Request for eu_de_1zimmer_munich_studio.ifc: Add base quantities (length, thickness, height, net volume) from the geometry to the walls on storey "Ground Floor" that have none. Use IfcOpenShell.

First a look at what the model holds.

```python
import ifcopenshell
import ifcopenshell.util.element
import ifcopenshell.util.unit

model = ifcopenshell.open("eu_de_1zimmer_munich_studio.ifc")
print(model.schema)
for unit_type in ("LENGTHUNIT", "AREAUNIT", "VOLUMEUNIT"):
    print(unit_type, ifcopenshell.util.unit.calculate_unit_scale(model, unit_type))
storey = next(s for s in model.by_type("IfcBuildingStorey") if s.Name == "Ground Floor")
walls = [e for e in ifcopenshell.util.element.get_decomposition(storey) if e.is_a("IfcWall")]
for e in sorted(walls, key=lambda e: e.id()):
    print(e.id(), e.is_a(), e.Name, list(ifcopenshell.util.element.get_psets(e, qtos_only=True)), sep=" | ")
```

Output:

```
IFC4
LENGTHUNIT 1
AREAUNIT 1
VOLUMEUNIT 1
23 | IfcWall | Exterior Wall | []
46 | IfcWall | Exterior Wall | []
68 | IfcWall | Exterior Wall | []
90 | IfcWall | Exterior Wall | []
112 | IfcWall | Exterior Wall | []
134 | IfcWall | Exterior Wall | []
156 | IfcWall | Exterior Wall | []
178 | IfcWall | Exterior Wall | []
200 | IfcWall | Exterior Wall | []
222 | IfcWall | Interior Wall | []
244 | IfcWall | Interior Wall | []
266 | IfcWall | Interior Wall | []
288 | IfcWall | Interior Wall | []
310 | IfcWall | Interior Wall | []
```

```python
import ifcopenshell
import ifcopenshell.api.pset
import ifcopenshell.geom
import ifcopenshell.util.element
import ifcopenshell.util.shape
import ifcopenshell.util.unit

model = ifcopenshell.open("eu_de_1zimmer_munich_studio.ifc")
unit_scale = ifcopenshell.util.unit.calculate_unit_scale(model)
volume_scale = ifcopenshell.util.unit.calculate_unit_scale(model, "VOLUMEUNIT")
settings = ifcopenshell.geom.settings()

storey = next(s for s in model.by_type("IfcBuildingStorey") if s.Name == "Ground Floor")
walls = [e for e in ifcopenshell.util.element.get_decomposition(storey) if e.is_a("IfcWall")]

for e in sorted(walls, key=lambda e: e.id()):
    if ifcopenshell.util.element.get_psets(e, qtos_only=True, should_inherit=False):
        continue
    # Geometry comes back in metres, in the element's own axes.
    shape = ifcopenshell.geom.create_shape(settings, e)
    values = {
        "Length": ifcopenshell.util.shape.get_x(shape.geometry) / unit_scale,
        "Width": ifcopenshell.util.shape.get_y(shape.geometry) / unit_scale,
        "Height": ifcopenshell.util.shape.get_z(shape.geometry) / unit_scale,
        "NetVolume": ifcopenshell.util.shape.get_volume(shape.geometry) / volume_scale,
    }
    qto = ifcopenshell.api.pset.add_qto(model, product=e, name="Qto_WallBaseQuantities")
    ifcopenshell.api.pset.edit_qto(model, qto=qto, properties=values)
    print(e.id(), {k: round(v, 3) for k, v in values.items()})

model.write("eu_de_1zimmer_munich_studio_edited.ifc")
```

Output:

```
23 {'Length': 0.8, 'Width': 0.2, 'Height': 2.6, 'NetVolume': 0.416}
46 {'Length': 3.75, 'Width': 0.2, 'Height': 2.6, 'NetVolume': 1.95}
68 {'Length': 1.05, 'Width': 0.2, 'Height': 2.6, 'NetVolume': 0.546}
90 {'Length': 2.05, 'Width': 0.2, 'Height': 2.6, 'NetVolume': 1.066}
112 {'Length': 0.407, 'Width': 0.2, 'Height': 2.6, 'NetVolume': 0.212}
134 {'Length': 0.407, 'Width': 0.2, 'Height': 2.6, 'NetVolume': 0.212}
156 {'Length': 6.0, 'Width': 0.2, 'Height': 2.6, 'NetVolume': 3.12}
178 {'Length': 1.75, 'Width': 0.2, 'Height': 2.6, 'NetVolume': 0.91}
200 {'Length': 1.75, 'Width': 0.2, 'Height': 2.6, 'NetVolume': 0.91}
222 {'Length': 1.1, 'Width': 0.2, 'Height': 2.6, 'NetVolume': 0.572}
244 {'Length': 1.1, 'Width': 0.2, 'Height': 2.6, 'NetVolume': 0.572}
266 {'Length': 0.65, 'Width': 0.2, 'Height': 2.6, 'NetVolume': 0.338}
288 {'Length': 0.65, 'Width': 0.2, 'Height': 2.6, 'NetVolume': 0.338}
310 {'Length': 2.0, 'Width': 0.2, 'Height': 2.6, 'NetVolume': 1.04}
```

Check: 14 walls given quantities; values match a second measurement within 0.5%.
